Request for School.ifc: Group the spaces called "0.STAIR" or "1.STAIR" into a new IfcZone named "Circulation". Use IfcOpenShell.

First a look at what the model holds.

```python
import ifcopenshell

model = ifcopenshell.open("School.ifc")
print(model.schema)
seen = {}
for space in model.by_type("IfcSpace"):
    seen[space.LongName] = seen.get(space.LongName, 0) + 1
for name, count in sorted(seen.items(), key=str):
    print(count, "x", name)
print("zones:", [z.Name for z in model.by_type("IfcZone")][:20])
```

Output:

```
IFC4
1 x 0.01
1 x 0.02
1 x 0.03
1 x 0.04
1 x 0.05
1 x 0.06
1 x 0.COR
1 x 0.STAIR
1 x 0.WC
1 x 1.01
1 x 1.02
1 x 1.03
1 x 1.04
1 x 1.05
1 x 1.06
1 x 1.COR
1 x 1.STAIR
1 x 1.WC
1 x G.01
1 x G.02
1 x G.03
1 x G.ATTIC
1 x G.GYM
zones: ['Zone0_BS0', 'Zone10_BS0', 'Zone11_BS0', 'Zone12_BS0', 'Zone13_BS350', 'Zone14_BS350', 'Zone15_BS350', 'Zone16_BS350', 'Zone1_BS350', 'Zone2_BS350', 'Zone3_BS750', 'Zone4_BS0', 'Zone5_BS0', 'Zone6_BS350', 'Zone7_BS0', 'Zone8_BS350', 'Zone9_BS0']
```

```python
import ifcopenshell
import ifcopenshell.api.group
import ifcopenshell.api.root

model = ifcopenshell.open("School.ifc")

names = {"0.STAIR", "1.STAIR"}
spaces = [s for s in model.by_type("IfcSpace") if s.LongName in names]

zone = ifcopenshell.api.root.create_entity(model, ifc_class="IfcZone", name="Circulation")
ifcopenshell.api.group.assign_group(model, products=spaces, group=zone)
print(len(spaces), "spaces in", zone.Name)

model.write("School_edited.ifc")
```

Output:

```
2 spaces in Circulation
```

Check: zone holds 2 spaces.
